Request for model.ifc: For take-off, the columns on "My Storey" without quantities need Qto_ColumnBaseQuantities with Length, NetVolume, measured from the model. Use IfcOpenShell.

First a look at what the model holds.

```python
import ifcopenshell
import ifcopenshell.util.element
import ifcopenshell.util.unit

model = ifcopenshell.open("model.ifc")
print(model.schema)
for unit_type in ("LENGTHUNIT", "AREAUNIT", "VOLUMEUNIT"):
    print(unit_type, ifcopenshell.util.unit.calculate_unit_scale(model, unit_type))
storey = next(s for s in model.by_type("IfcBuildingStorey") if s.Name == "My Storey")
columns = [e for e in ifcopenshell.util.element.get_decomposition(storey) if e.is_a("IfcColumn")]
for e in sorted(columns, key=lambda e: e.id()):
    print(e.id(), e.is_a(), e.Name, list(ifcopenshell.util.element.get_psets(e, qtos_only=True)), sep=" | ")
```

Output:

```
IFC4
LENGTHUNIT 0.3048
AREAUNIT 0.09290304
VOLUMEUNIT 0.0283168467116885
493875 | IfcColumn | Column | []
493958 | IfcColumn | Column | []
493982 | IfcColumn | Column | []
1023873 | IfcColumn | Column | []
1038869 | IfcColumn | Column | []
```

```python
import ifcopenshell
import ifcopenshell.api.pset
import ifcopenshell.geom
import ifcopenshell.util.element
import ifcopenshell.util.shape
import ifcopenshell.util.unit

model = ifcopenshell.open("model.ifc")
unit_scale = ifcopenshell.util.unit.calculate_unit_scale(model)
volume_scale = ifcopenshell.util.unit.calculate_unit_scale(model, "VOLUMEUNIT")
settings = ifcopenshell.geom.settings()

storey = next(s for s in model.by_type("IfcBuildingStorey") if s.Name == "My Storey")
columns = [e for e in ifcopenshell.util.element.get_decomposition(storey) if e.is_a("IfcColumn")]

for e in sorted(columns, key=lambda e: e.id()):
    if ifcopenshell.util.element.get_psets(e, qtos_only=True, should_inherit=False):
        continue
    # Geometry comes back in metres, in the element's own axes.
    shape = ifcopenshell.geom.create_shape(settings, e)
    values = {
        "Length": ifcopenshell.util.shape.get_z(shape.geometry) / unit_scale,
        "NetVolume": ifcopenshell.util.shape.get_volume(shape.geometry) / volume_scale,
    }
    qto = ifcopenshell.api.pset.add_qto(model, product=e, name="Qto_ColumnBaseQuantities")
    ifcopenshell.api.pset.edit_qto(model, qto=qto, properties=values)
    print(e.id(), {k: round(v, 3) for k, v in values.items()})

model.write("model_edited.ifc")
```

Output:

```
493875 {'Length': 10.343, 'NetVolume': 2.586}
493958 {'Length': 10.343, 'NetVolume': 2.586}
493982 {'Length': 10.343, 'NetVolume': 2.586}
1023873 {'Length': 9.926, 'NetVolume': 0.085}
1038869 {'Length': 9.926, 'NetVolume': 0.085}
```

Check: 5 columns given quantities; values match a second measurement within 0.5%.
